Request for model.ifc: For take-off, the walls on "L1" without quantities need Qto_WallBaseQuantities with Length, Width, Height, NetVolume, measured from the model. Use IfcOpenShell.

First a look at what the model holds.

```python
import ifcopenshell
import ifcopenshell.util.element
import ifcopenshell.util.unit

model = ifcopenshell.open("model.ifc")
print(model.schema)
for unit_type in ("LENGTHUNIT", "AREAUNIT", "VOLUMEUNIT"):
    print(unit_type, ifcopenshell.util.unit.calculate_unit_scale(model, unit_type))
storey = next(s for s in model.by_type("IfcBuildingStorey") if s.Name == "L1")
walls = [e for e in ifcopenshell.util.element.get_decomposition(storey) if e.is_a("IfcWall")]
for e in sorted(walls, key=lambda e: e.id()):
    print(e.id(), e.is_a(), e.Name, list(ifcopenshell.util.element.get_psets(e, qtos_only=True)), sep=" | ")
```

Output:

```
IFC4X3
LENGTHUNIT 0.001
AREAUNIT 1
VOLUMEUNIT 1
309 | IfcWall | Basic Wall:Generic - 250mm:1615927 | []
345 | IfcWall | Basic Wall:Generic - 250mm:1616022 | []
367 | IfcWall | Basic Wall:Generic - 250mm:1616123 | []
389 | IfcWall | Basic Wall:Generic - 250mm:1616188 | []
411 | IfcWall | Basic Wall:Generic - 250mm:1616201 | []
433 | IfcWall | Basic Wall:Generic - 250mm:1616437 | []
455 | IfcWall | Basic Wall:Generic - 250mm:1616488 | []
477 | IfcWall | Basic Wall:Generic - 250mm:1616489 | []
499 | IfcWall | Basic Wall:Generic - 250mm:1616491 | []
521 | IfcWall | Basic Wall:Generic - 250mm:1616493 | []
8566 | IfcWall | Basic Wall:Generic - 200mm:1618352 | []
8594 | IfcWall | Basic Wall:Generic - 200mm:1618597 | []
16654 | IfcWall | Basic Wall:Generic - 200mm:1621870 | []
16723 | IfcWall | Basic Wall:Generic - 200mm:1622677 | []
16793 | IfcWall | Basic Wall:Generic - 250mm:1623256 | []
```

```python
import ifcopenshell
import ifcopenshell.api.pset
import ifcopenshell.geom
import ifcopenshell.util.element
import ifcopenshell.util.shape
import ifcopenshell.util.unit

model = ifcopenshell.open("model.ifc")
unit_scale = ifcopenshell.util.unit.calculate_unit_scale(model)
volume_scale = ifcopenshell.util.unit.calculate_unit_scale(model, "VOLUMEUNIT")
settings = ifcopenshell.geom.settings()

storey = next(s for s in model.by_type("IfcBuildingStorey") if s.Name == "L1")
walls = [e for e in ifcopenshell.util.element.get_decomposition(storey) if e.is_a("IfcWall")]

for e in sorted(walls, key=lambda e: e.id()):
    if ifcopenshell.util.element.get_psets(e, qtos_only=True, should_inherit=False):
        continue
    # Geometry comes back in metres, in the element's own axes.
    shape = ifcopenshell.geom.create_shape(settings, e)
    values = {
        "Length": ifcopenshell.util.shape.get_x(shape.geometry) / unit_scale,
        "Width": ifcopenshell.util.shape.get_y(shape.geometry) / unit_scale,
        "Height": ifcopenshell.util.shape.get_z(shape.geometry) / unit_scale,
        "NetVolume": ifcopenshell.util.shape.get_volume(shape.geometry) / volume_scale,
    }
    qto = ifcopenshell.api.pset.add_qto(model, product=e, name="Qto_WallBaseQuantities")
    ifcopenshell.api.pset.edit_qto(model, qto=qto, properties=values)
    print(e.id(), {k: round(v, 3) for k, v in values.items()})

model.write("model_rev.ifc")
```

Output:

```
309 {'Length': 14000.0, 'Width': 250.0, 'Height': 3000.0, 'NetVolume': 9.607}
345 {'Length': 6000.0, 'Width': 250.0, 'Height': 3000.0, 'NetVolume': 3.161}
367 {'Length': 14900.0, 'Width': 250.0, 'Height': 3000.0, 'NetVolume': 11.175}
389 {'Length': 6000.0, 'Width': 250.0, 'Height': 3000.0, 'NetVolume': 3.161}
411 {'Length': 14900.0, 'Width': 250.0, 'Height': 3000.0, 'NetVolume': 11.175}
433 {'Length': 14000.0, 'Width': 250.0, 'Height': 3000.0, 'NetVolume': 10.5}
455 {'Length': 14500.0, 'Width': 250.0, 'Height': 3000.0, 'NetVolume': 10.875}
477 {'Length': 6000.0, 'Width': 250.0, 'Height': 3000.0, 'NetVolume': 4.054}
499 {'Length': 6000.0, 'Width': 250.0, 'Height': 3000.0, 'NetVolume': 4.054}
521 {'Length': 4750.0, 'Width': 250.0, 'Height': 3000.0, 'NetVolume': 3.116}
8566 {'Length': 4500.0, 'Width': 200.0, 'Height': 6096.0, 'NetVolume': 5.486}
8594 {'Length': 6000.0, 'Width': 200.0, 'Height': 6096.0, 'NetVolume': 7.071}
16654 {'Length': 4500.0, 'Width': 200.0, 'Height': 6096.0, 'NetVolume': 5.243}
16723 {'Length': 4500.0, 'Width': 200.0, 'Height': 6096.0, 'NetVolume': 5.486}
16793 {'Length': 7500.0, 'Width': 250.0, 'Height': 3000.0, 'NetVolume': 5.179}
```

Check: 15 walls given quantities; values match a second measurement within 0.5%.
